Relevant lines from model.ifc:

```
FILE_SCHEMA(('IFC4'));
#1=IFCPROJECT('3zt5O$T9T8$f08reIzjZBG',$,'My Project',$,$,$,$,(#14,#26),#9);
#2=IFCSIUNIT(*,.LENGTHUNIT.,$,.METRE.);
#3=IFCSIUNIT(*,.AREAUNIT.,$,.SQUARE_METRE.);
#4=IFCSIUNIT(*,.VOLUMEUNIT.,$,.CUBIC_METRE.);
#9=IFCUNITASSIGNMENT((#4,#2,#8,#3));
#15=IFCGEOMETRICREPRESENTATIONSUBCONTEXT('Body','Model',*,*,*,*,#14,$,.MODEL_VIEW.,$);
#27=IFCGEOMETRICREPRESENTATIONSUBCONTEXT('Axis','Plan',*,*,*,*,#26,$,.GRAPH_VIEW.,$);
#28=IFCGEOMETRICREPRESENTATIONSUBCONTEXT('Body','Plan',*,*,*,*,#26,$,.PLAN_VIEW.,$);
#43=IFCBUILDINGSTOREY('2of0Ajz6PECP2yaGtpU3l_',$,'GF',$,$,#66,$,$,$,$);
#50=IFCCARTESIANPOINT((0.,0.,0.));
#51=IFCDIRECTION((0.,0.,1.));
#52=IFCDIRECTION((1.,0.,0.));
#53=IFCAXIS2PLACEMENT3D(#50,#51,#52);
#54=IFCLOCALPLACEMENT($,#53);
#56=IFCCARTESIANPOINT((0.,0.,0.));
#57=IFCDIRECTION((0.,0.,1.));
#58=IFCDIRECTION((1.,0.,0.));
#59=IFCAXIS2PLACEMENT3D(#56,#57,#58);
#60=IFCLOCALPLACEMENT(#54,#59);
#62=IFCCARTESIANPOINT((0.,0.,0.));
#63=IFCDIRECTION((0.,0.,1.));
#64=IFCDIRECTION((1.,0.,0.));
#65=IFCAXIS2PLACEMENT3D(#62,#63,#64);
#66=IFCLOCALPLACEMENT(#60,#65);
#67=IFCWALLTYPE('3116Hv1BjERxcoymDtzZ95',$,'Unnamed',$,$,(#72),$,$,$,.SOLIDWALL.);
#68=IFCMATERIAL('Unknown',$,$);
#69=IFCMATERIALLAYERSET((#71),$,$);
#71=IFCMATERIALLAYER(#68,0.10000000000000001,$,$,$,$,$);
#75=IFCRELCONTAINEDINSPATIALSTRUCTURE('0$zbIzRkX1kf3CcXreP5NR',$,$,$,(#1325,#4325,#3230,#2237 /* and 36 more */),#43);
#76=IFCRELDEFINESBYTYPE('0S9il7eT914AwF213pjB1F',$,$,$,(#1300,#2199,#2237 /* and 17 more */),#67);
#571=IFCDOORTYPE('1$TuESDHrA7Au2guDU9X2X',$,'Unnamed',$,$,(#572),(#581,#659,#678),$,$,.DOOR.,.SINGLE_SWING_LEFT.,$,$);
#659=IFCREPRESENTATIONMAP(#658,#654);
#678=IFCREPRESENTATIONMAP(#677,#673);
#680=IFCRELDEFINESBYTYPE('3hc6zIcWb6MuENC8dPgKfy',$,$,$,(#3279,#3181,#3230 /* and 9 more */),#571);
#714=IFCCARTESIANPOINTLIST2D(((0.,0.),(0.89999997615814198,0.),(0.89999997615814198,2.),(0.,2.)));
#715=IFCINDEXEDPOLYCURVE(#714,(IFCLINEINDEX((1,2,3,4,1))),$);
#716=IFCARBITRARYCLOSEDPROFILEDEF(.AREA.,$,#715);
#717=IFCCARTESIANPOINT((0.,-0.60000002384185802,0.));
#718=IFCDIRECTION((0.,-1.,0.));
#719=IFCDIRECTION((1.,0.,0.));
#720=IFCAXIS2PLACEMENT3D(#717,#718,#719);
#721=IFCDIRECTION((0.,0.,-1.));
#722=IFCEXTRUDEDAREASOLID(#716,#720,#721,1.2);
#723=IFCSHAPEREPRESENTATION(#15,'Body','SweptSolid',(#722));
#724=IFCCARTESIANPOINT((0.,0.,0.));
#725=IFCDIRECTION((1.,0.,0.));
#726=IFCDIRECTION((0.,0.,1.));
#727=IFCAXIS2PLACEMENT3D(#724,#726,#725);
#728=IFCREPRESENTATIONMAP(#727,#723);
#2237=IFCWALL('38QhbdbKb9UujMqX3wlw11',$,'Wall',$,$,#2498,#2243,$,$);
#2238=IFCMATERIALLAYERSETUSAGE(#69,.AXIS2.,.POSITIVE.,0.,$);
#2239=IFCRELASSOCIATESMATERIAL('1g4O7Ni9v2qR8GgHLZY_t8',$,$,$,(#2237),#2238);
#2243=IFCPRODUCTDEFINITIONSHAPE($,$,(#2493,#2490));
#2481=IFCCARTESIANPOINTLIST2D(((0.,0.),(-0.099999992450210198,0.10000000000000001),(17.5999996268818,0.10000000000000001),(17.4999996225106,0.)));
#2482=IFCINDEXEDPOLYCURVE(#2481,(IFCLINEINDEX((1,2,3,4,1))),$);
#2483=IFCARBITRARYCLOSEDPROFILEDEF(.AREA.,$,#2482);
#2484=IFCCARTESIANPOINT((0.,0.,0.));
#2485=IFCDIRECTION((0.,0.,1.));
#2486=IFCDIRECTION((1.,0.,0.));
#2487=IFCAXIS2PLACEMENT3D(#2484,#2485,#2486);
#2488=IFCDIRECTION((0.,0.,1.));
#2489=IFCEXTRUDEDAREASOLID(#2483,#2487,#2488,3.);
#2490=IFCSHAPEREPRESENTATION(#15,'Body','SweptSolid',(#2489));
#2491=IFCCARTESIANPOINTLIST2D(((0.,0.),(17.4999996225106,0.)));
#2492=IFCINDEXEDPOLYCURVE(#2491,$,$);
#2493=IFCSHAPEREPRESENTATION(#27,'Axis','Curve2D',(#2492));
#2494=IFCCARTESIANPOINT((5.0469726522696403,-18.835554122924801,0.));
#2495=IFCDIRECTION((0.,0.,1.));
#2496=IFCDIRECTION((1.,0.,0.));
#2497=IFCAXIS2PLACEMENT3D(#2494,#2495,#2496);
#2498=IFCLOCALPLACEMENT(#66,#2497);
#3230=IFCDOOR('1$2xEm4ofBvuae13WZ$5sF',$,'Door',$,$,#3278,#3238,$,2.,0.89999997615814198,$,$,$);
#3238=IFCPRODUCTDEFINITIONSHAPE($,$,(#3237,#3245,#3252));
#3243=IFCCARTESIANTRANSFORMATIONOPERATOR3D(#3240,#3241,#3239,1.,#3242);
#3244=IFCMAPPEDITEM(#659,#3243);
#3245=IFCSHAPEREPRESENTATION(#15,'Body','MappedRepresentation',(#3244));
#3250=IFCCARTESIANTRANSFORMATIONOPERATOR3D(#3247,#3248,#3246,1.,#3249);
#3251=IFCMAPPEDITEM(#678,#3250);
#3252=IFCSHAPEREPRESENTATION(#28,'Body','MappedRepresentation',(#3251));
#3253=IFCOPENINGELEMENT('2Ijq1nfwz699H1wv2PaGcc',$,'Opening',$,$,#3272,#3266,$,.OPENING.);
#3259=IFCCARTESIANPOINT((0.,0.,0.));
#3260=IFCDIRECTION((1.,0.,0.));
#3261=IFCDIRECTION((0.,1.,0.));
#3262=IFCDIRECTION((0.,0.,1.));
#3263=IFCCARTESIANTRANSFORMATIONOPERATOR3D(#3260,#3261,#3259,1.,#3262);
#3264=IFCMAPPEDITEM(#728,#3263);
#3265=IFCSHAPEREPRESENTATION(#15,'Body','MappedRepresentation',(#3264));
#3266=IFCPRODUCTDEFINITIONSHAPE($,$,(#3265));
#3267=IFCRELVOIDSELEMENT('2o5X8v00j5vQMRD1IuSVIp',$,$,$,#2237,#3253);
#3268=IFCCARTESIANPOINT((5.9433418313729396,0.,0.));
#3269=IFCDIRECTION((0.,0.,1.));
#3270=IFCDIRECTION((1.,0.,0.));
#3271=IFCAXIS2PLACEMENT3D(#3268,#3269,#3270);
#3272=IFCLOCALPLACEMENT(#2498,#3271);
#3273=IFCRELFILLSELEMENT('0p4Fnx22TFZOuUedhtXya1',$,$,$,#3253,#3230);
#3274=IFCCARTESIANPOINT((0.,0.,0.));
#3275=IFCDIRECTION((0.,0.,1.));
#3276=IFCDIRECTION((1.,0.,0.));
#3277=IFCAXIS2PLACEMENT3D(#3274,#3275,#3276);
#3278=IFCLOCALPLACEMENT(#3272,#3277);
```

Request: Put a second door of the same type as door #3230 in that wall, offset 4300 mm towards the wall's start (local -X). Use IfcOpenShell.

```python
import ifcopenshell
import ifcopenshell.api.feature
import ifcopenshell.api.geometry
import ifcopenshell.api.root
import ifcopenshell.geom
import ifcopenshell.util.element
import ifcopenshell.util.placement
import ifcopenshell.util.shape
import ifcopenshell.util.unit

model = ifcopenshell.open("model.ifc")
unit_scale = ifcopenshell.util.unit.calculate_unit_scale(model)
settings = ifcopenshell.geom.settings()


def volume(element):
    """Net volume in cubic metres, openings subtracted."""
    shape = ifcopenshell.geom.create_shape(settings, element)
    return ifcopenshell.util.shape.get_volume(shape.geometry)


door = model.by_guid("1$2xEm4ofBvuae13WZ$5sF")
opening = door.FillsVoids[0].RelatingOpeningElement
wall = opening.VoidsElements[0].RelatingBuildingElement
before = volume(wall)
shift = ifcopenshell.util.placement.get_local_placement(wall.ObjectPlacement)[:3, 0] * -4.3 / unit_scale

# copy_class copies the void relationship, type, container and properties, but no geometry.
new_opening = ifcopenshell.api.root.copy_class(model, product=opening)
new_opening.Representation = ifcopenshell.util.element.copy_deep(
    model, opening.Representation, exclude=["IfcGeometricRepresentationContext", "IfcRepresentationMap"]
)
new_door = ifcopenshell.api.root.copy_class(model, product=door)
new_door.Representation = ifcopenshell.util.element.copy_deep(
    model, door.Representation, exclude=["IfcGeometricRepresentationContext", "IfcRepresentationMap"]
)
ifcopenshell.api.feature.add_filling(model, opening=new_opening, element=new_door)

for old, new in ((opening, new_opening), (door, new_door)):
    matrix = ifcopenshell.util.placement.get_local_placement(old.ObjectPlacement)
    matrix[:3, 3] += shift
    ifcopenshell.api.geometry.edit_object_placement(model, product=new, matrix=matrix, is_si=False)

after = volume(wall)

print(f"wall volume {before:.3f} -> {after:.3f} m3")

model.write("model_v2.ifc")
```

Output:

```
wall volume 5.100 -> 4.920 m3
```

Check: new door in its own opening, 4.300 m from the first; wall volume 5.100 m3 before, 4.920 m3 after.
